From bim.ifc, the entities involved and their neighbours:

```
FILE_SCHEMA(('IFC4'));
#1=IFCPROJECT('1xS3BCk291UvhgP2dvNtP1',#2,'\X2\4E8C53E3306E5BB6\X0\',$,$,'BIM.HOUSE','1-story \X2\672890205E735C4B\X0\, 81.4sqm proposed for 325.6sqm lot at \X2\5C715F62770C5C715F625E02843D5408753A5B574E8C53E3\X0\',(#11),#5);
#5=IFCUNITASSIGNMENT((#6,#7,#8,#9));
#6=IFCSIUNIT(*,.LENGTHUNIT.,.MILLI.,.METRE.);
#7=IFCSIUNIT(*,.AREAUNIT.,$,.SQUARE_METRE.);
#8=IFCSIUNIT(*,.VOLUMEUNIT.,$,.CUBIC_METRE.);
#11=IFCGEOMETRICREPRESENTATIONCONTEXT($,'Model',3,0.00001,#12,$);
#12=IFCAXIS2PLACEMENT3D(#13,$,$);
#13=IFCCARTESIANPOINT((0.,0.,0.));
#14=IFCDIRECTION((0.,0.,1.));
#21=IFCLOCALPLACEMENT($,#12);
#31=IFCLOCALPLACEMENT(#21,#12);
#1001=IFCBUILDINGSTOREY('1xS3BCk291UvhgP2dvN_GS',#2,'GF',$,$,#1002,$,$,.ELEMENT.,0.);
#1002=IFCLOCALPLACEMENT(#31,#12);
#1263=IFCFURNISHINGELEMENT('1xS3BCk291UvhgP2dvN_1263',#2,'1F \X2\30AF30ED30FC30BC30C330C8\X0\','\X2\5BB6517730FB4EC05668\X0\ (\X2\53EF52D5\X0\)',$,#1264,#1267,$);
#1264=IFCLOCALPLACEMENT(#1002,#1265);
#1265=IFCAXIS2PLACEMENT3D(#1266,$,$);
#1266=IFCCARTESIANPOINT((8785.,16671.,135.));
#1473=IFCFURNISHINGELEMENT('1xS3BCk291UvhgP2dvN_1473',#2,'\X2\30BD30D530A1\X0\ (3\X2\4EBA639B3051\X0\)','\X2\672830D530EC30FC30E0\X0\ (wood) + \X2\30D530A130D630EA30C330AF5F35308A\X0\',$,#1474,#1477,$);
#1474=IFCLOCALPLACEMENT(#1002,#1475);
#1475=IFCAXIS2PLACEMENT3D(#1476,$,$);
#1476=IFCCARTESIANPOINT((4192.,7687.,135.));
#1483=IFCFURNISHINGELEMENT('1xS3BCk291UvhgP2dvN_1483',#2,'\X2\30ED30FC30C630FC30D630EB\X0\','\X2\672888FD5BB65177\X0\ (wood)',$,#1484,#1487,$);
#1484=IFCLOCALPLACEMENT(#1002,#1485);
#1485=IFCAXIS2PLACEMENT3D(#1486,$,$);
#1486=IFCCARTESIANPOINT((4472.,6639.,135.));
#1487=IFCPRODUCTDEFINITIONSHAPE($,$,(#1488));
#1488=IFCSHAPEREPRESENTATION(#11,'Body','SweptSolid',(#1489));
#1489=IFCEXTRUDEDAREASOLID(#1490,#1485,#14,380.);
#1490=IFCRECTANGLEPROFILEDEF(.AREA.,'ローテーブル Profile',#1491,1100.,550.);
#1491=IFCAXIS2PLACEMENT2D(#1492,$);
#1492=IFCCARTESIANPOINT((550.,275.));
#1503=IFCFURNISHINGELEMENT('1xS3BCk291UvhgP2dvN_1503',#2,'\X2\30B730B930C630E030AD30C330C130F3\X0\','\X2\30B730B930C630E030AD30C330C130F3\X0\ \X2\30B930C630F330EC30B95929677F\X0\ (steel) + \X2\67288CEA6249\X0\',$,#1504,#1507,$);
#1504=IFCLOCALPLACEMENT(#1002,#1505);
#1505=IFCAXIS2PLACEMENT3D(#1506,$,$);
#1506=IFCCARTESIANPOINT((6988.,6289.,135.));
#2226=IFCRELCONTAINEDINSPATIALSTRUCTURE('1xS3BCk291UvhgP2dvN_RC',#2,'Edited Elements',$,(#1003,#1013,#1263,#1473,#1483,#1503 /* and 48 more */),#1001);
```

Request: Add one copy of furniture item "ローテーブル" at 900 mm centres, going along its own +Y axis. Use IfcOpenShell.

```python
import ifcopenshell
import ifcopenshell.api.geometry
import ifcopenshell.api.root
import ifcopenshell.util.element
import ifcopenshell.util.placement

model = ifcopenshell.open("bim.ifc")


def reuse_history(source, copy):
    """copy_class also copies each property set's owner history, people and application; keep the originals."""
    for rel in copy.IsDefinedBy:
        if rel.is_a("IfcRelDefinesByProperties") and (history := rel.RelatingPropertyDefinition.OwnerHistory):
            rel.RelatingPropertyDefinition.OwnerHistory = source.OwnerHistory
            ifcopenshell.util.element.remove_deep2(model, history)


source = model.by_guid("1xS3BCk291UvhgP2dvN_1483")
base = ifcopenshell.util.placement.get_local_placement(source.ObjectPlacement)
step = base[:3, 1] * 900.0

for i in range(1, 2):
    copy = ifcopenshell.api.root.copy_class(model, product=source)
    copy.Representation = ifcopenshell.util.element.copy_deep(
        model, source.Representation, exclude=["IfcGeometricRepresentationContext", "IfcRepresentationMap"]
    )
    reuse_history(source, copy)
    matrix = base.copy()
    matrix[:3, 3] += i * step
    print("added at", matrix[:3, 3].round(3) + 0.0)
    ifcopenshell.api.geometry.edit_object_placement(model, product=copy, matrix=matrix, is_si=False)

model.write("bim_updated.ifc")
```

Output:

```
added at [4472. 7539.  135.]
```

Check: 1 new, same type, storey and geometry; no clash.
